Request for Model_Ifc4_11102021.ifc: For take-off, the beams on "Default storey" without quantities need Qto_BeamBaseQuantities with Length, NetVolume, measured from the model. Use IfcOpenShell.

First a look at what the model holds.

```python
import ifcopenshell
import ifcopenshell.util.element
import ifcopenshell.util.unit

model = ifcopenshell.open("Model_Ifc4_11102021.ifc")
print(model.schema)
for unit_type in ("LENGTHUNIT", "AREAUNIT", "VOLUMEUNIT"):
    print(unit_type, ifcopenshell.util.unit.calculate_unit_scale(model, unit_type))
storey = next(s for s in model.by_type("IfcBuildingStorey") if s.Name == "Default storey")
beams = [e for e in ifcopenshell.util.element.get_decomposition(storey) if e.is_a("IfcBeam")]
for e in sorted(beams, key=lambda e: e.id()):
    print(e.id(), e.is_a(), e.Name, list(ifcopenshell.util.element.get_psets(e, qtos_only=True)), sep=" | ")
```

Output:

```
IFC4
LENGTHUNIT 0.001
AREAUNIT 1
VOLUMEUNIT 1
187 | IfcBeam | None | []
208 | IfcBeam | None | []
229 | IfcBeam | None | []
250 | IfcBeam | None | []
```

```python
import ifcopenshell
import ifcopenshell.api.pset
import ifcopenshell.geom
import ifcopenshell.util.element
import ifcopenshell.util.shape
import ifcopenshell.util.unit

model = ifcopenshell.open("Model_Ifc4_11102021.ifc")
unit_scale = ifcopenshell.util.unit.calculate_unit_scale(model)
volume_scale = ifcopenshell.util.unit.calculate_unit_scale(model, "VOLUMEUNIT")
settings = ifcopenshell.geom.settings()

storey = next(s for s in model.by_type("IfcBuildingStorey") if s.Name == "Default storey")
beams = [e for e in ifcopenshell.util.element.get_decomposition(storey) if e.is_a("IfcBeam")]

for e in sorted(beams, key=lambda e: e.id()):
    if ifcopenshell.util.element.get_psets(e, qtos_only=True, should_inherit=False):
        continue
    # Geometry comes back in metres, in the element's own axes.
    shape = ifcopenshell.geom.create_shape(settings, e)
    values = {
        "Length": ifcopenshell.util.shape.get_max_xyz(shape.geometry) / unit_scale,
        "NetVolume": ifcopenshell.util.shape.get_volume(shape.geometry) / volume_scale,
    }
    qto = ifcopenshell.api.pset.add_qto(model, product=e, name="Qto_BeamBaseQuantities")
    ifcopenshell.api.pset.edit_qto(model, qto=qto, properties=values)
    print(e.id(), {k: round(v, 3) for k, v in values.items()})

model.write("Model_Ifc4_11102021_updated.ifc")
```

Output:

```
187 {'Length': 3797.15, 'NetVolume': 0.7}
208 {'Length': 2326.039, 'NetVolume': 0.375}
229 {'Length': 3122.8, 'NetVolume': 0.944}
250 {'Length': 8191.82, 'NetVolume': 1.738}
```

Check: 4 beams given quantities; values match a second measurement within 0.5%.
